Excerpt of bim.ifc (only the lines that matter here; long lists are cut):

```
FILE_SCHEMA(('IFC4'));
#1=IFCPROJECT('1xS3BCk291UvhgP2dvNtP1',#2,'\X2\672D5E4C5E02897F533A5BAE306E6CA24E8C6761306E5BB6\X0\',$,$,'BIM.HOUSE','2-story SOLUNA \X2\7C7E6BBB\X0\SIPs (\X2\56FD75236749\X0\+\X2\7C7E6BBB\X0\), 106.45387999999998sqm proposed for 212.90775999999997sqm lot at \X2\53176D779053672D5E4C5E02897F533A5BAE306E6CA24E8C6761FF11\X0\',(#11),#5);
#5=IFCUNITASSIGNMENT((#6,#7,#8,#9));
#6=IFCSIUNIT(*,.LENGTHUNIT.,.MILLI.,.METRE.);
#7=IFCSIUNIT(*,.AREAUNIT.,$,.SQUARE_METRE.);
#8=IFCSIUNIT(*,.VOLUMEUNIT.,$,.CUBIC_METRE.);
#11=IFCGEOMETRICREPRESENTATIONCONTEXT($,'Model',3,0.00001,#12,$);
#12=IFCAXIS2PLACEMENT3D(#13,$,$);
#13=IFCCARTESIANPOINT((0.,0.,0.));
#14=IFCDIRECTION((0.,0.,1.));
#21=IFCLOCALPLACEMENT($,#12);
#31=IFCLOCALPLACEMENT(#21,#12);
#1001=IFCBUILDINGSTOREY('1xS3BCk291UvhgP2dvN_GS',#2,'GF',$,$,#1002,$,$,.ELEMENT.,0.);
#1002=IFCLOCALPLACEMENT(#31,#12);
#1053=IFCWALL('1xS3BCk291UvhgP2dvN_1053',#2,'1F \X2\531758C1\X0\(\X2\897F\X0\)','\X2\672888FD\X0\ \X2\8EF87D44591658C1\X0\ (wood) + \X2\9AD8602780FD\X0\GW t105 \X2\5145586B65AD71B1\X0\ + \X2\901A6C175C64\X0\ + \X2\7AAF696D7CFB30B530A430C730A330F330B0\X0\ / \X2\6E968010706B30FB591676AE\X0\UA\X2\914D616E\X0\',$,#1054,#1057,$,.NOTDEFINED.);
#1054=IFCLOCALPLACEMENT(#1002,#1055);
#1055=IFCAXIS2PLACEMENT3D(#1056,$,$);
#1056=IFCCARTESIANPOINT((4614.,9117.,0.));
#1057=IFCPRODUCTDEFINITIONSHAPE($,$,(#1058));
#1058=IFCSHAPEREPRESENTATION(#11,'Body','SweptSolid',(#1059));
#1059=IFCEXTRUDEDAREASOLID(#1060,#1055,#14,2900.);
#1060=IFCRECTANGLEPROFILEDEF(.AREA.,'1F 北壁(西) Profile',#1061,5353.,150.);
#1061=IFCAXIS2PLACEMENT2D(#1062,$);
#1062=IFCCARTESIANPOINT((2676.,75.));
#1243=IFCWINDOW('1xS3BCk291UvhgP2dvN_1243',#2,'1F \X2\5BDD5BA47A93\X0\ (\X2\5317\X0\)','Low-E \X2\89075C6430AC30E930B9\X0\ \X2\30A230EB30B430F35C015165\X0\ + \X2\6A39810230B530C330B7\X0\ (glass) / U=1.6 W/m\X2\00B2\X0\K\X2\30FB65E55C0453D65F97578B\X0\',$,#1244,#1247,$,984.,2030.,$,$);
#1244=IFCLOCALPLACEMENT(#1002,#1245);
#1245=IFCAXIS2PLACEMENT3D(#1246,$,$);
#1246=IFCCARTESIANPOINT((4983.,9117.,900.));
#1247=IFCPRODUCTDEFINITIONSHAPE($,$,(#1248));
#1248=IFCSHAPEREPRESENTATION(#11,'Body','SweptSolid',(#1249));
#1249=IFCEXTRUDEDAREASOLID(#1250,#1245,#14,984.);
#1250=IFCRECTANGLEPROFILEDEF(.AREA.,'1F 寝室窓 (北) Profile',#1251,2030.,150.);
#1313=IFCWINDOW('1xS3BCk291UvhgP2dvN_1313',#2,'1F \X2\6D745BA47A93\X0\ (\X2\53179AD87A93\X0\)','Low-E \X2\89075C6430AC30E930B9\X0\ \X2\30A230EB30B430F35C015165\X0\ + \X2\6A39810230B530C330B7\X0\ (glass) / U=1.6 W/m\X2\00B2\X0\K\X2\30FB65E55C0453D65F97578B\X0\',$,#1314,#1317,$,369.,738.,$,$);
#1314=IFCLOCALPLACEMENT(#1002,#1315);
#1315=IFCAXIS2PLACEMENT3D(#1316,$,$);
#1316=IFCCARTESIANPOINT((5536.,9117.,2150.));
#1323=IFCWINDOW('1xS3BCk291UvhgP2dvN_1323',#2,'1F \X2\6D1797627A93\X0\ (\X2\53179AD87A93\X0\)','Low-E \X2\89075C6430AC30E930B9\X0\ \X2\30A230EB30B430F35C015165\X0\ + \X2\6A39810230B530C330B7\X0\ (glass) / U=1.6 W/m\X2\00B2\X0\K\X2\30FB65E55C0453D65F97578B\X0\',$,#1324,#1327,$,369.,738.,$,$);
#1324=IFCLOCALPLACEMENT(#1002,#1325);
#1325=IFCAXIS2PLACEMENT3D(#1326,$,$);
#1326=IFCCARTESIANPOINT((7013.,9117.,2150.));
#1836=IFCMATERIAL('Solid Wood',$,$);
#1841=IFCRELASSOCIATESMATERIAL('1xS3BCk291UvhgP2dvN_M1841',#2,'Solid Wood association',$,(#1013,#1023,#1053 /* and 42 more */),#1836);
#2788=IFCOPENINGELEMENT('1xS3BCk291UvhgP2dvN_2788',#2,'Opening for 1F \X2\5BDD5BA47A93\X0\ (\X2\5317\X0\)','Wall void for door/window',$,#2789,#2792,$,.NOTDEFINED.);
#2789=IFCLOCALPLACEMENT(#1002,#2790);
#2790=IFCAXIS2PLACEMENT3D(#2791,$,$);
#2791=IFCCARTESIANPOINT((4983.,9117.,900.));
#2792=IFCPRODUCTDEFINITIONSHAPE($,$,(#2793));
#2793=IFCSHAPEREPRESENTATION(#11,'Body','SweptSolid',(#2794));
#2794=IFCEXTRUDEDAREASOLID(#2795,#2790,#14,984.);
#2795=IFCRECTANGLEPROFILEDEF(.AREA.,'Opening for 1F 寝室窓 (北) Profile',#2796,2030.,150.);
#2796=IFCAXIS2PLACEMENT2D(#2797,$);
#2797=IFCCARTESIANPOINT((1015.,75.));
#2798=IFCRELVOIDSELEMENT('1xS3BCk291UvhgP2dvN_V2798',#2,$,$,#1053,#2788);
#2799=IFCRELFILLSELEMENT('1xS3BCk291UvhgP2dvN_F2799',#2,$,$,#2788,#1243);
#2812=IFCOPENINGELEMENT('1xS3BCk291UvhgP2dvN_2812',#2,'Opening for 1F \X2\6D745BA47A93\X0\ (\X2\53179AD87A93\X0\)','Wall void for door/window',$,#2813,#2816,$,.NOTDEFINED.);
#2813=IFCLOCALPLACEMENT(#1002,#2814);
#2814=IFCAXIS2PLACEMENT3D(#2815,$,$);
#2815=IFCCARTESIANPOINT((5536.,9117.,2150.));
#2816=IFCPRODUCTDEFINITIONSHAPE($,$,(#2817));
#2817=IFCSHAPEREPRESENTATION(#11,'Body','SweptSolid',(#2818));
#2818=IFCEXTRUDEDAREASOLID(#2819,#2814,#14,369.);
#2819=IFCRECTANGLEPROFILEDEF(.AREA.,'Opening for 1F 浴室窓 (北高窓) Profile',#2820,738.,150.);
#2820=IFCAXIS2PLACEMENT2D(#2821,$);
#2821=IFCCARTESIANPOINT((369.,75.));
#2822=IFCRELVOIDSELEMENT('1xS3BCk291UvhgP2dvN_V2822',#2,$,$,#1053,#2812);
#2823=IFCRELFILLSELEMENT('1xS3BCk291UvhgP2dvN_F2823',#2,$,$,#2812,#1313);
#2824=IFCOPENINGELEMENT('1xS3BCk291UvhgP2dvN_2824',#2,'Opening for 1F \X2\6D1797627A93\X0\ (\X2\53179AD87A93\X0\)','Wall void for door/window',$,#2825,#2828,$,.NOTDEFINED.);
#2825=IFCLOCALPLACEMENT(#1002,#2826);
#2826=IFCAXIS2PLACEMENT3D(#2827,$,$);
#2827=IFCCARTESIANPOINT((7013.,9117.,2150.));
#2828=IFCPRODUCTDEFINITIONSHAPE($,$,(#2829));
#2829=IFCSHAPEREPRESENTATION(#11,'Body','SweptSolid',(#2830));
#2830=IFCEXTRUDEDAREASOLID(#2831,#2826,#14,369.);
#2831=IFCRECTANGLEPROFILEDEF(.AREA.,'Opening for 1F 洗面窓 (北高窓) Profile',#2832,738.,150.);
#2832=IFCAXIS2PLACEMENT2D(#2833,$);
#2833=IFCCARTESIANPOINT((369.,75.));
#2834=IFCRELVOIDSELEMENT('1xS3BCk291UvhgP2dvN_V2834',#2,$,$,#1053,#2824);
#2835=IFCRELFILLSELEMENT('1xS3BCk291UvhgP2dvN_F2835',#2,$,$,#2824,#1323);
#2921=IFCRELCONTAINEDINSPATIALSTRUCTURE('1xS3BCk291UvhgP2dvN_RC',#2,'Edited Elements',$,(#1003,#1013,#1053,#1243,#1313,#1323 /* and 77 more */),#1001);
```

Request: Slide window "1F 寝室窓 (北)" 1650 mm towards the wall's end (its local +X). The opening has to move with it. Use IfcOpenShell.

```python
import ifcopenshell
import ifcopenshell.api.geometry
import ifcopenshell.util.placement

model = ifcopenshell.open("bim.ifc")

window = model.by_guid("1xS3BCk291UvhgP2dvN_1243")
opening = window.FillsVoids[0].RelatingOpeningElement
wall = opening.VoidsElements[0].RelatingBuildingElement

wall_matrix = ifcopenshell.util.placement.get_local_placement(wall.ObjectPlacement)
shift = wall_matrix[:3, 0] * 1650.0
before = ifcopenshell.util.placement.get_local_placement(window.ObjectPlacement)[:3, 3].copy()

# The window is not placed relative to its opening, so move both.
for product in (opening, window):
    matrix = ifcopenshell.util.placement.get_local_placement(product.ObjectPlacement)
    matrix[:3, 3] += shift
    ifcopenshell.api.geometry.edit_object_placement(model, product=product, matrix=matrix, is_si=False)

after = ifcopenshell.util.placement.get_local_placement(window.ObjectPlacement)[:3, 3]
print("window moved by", (after - before).round(3) + 0.0)

model.write("bim_rev.ifc")
```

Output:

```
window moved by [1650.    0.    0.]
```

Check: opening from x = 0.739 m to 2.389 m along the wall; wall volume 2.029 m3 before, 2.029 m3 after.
